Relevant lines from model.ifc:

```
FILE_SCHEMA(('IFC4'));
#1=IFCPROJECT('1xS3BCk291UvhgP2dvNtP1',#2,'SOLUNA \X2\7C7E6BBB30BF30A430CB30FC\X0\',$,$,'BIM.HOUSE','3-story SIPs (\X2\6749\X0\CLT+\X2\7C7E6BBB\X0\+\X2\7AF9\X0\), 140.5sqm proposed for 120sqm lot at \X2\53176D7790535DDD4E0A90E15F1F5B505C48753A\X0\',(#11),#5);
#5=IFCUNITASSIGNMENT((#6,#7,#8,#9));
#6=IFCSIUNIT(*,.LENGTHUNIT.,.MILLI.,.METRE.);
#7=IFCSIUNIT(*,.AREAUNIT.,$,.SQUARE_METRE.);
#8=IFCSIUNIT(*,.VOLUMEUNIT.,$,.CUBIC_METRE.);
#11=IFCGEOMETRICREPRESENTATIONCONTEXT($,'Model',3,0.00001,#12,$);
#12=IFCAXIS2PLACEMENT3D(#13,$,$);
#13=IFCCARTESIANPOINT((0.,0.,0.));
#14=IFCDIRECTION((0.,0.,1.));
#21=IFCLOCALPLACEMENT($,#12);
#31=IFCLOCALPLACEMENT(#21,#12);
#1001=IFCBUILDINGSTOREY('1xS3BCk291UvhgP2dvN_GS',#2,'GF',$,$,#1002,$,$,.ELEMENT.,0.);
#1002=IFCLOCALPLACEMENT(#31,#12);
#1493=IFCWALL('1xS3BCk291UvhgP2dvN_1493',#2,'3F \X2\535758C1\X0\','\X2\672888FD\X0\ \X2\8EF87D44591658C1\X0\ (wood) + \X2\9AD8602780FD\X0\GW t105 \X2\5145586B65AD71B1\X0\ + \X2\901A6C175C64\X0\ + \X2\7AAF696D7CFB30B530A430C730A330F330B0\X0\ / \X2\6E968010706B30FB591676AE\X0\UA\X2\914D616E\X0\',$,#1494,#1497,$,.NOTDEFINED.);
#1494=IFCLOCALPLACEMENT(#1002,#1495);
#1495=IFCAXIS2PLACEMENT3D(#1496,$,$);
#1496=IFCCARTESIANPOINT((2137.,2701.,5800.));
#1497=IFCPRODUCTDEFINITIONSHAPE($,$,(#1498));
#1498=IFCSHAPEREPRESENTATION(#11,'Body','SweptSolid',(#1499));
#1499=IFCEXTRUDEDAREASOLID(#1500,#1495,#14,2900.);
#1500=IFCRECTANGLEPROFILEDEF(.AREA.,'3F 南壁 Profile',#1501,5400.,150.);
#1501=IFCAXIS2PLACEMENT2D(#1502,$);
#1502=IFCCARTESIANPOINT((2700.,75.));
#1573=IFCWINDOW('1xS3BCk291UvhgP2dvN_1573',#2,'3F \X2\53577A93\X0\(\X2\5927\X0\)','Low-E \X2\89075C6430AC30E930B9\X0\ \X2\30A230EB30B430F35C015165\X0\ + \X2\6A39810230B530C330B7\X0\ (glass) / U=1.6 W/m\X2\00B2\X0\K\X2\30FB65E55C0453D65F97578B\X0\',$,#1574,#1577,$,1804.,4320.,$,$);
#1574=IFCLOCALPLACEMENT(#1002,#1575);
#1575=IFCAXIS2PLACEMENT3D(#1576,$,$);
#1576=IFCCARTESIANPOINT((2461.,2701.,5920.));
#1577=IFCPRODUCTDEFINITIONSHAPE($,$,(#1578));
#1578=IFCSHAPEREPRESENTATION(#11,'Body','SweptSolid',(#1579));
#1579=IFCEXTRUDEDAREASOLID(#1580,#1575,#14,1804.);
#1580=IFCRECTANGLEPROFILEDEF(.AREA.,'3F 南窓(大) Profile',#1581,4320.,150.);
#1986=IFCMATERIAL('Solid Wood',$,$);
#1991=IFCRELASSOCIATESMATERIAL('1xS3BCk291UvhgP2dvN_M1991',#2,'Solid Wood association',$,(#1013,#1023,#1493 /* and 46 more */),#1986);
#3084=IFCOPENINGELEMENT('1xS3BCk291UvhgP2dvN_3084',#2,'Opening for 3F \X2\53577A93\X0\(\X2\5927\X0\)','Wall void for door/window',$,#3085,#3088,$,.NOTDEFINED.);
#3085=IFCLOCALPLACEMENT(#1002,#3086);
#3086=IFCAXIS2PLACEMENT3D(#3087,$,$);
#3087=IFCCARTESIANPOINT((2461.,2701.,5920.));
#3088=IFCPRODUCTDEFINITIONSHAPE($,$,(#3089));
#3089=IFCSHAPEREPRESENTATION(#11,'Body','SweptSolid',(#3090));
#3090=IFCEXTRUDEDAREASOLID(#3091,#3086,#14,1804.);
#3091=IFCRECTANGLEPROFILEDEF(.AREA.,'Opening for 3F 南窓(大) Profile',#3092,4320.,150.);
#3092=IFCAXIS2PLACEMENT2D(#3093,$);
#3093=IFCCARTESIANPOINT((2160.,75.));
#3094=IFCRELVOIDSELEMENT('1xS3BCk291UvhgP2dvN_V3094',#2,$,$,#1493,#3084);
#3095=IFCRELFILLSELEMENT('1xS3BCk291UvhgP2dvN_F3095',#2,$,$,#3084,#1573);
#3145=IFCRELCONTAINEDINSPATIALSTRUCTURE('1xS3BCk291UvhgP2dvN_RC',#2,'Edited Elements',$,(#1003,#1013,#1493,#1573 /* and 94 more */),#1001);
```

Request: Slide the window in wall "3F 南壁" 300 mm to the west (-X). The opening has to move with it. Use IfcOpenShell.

```python
import ifcopenshell
import ifcopenshell.api.geometry
import ifcopenshell.util.placement

model = ifcopenshell.open("model.ifc")

window = model.by_guid("1xS3BCk291UvhgP2dvN_1573")
opening = window.FillsVoids[0].RelatingOpeningElement
wall = opening.VoidsElements[0].RelatingBuildingElement

wall_matrix = ifcopenshell.util.placement.get_local_placement(wall.ObjectPlacement)
shift = wall_matrix[:3, 0] * -300.0
before = ifcopenshell.util.placement.get_local_placement(window.ObjectPlacement)[:3, 3].copy()

# The window is not placed relative to its opening, so move both.
for product in (opening, window):
    matrix = ifcopenshell.util.placement.get_local_placement(product.ObjectPlacement)
    matrix[:3, 3] += shift
    ifcopenshell.api.geometry.edit_object_placement(model, product=product, matrix=matrix, is_si=False)

after = ifcopenshell.util.placement.get_local_placement(window.ObjectPlacement)[:3, 3]
print("window moved by", (after - before).round(3) + 0.0)

model.write("model-out.ifc")
```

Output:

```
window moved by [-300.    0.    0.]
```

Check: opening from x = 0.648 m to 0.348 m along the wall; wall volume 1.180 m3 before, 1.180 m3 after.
